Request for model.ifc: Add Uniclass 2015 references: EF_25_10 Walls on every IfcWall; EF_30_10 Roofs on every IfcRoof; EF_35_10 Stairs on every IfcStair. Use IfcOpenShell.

First a look at what the model holds.

```python
import ifcopenshell

model = ifcopenshell.open("model.ifc")
print(model.schema)
print("classifications:", [c.Name for c in model.by_type("IfcClassification")])
for ifc_class in ("IfcDoor", "IfcRoof", "IfcStair", "IfcWall", "IfcWindow"):
    print(ifc_class, len(model.by_type(ifc_class)))
```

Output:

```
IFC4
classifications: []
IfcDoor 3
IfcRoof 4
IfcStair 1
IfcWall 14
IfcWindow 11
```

```python
import ifcopenshell
import ifcopenshell.api.classification

model = ifcopenshell.open("model.ifc")

system = ifcopenshell.api.classification.add_classification(model, classification="Uniclass 2015")

codes = {
    "IfcWall": ("EF_25_10", "Walls"),
    "IfcRoof": ("EF_30_10", "Roofs"),
    "IfcStair": ("EF_35_10", "Stairs"),
}
for ifc_class, (code, name) in codes.items():
    products = model.by_type(ifc_class)
    ifcopenshell.api.classification.add_reference(
        model, products=products, classification=system, identification=code, name=name
    )
    print(code, len(products))

model.write("model_v2.ifc")
```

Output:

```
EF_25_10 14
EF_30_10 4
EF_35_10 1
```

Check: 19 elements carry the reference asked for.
